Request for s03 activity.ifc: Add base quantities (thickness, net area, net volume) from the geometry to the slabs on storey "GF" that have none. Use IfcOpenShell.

First a look at what the model holds.

```python
import ifcopenshell
import ifcopenshell.util.element
import ifcopenshell.util.unit

model = ifcopenshell.open("s03 activity.ifc")
print(model.schema)
for unit_type in ("LENGTHUNIT", "AREAUNIT", "VOLUMEUNIT"):
    print(unit_type, ifcopenshell.util.unit.calculate_unit_scale(model, unit_type))
storey = next(s for s in model.by_type("IfcBuildingStorey") if s.Name == "GF")
slabs = [e for e in ifcopenshell.util.element.get_decomposition(storey) if e.is_a("IfcSlab")]
for e in sorted(slabs, key=lambda e: e.id()):
    print(e.id(), e.is_a(), e.Name, list(ifcopenshell.util.element.get_psets(e, qtos_only=True)), sep=" | ")
```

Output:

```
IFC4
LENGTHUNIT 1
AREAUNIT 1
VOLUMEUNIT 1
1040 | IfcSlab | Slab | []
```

```python
import ifcopenshell
import ifcopenshell.api.pset
import ifcopenshell.geom
import ifcopenshell.util.element
import ifcopenshell.util.shape
import ifcopenshell.util.unit

model = ifcopenshell.open("s03 activity.ifc")
unit_scale = ifcopenshell.util.unit.calculate_unit_scale(model)
area_scale = ifcopenshell.util.unit.calculate_unit_scale(model, "AREAUNIT")
volume_scale = ifcopenshell.util.unit.calculate_unit_scale(model, "VOLUMEUNIT")
settings = ifcopenshell.geom.settings()

storey = next(s for s in model.by_type("IfcBuildingStorey") if s.Name == "GF")
slabs = [e for e in ifcopenshell.util.element.get_decomposition(storey) if e.is_a("IfcSlab")]

for e in sorted(slabs, key=lambda e: e.id()):
    if ifcopenshell.util.element.get_psets(e, qtos_only=True, should_inherit=False):
        continue
    # Geometry comes back in metres, in the element's own axes.
    shape = ifcopenshell.geom.create_shape(settings, e)
    values = {
        "Width": ifcopenshell.util.shape.get_z(shape.geometry) / unit_scale,
        "NetArea": ifcopenshell.util.shape.get_footprint_area(shape.geometry) / area_scale,
        "NetVolume": ifcopenshell.util.shape.get_volume(shape.geometry) / volume_scale,
    }
    qto = ifcopenshell.api.pset.add_qto(model, product=e, name="Qto_SlabBaseQuantities")
    ifcopenshell.api.pset.edit_qto(model, qto=qto, properties=values)
    print(e.id(), {k: round(v, 3) for k, v in values.items()})

model.write("s03 activity_updated.ifc")
```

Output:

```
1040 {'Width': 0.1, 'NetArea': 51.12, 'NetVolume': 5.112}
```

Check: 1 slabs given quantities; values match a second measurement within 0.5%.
